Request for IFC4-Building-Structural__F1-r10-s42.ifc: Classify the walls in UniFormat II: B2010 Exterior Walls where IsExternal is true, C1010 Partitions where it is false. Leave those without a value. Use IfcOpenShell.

First a look at what the model holds.

```python
import ifcopenshell
import ifcopenshell.util.element

model = ifcopenshell.open("IFC4-Building-Structural__F1-r10-s42.ifc")
print(model.schema)
print("classifications:", [c.Name for c in model.by_type("IfcClassification")])
values = [ifcopenshell.util.element.get_pset(e, "Pset_WallCommon", "IsExternal") for e in model.by_type("IfcWall")]
for value in (True, False, None):
    print("IsExternal", value, values.count(value))
```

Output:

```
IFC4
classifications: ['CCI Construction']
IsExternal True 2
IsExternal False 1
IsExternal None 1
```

```python
import ifcopenshell
import ifcopenshell.api.classification
import ifcopenshell.util.element

model = ifcopenshell.open("IFC4-Building-Structural__F1-r10-s42.ifc")

system = ifcopenshell.api.classification.add_classification(model, classification="UniFormat II")

walls = model.by_type("IfcWall")
external = {e: ifcopenshell.util.element.get_pset(e, "Pset_WallCommon", "IsExternal") for e in walls}
for flag, code, name in ((True, "B2010", "Exterior Walls"), (False, "C1010", "Partitions")):
    products = [e for e in walls if external[e] is flag]
    ifcopenshell.api.classification.add_reference(
        model, products=products, classification=system, identification=code, name=name
    )
    print(code, len(products))

model.write("IFC4-Building-Structural__F1-r10-s42-out.ifc")
```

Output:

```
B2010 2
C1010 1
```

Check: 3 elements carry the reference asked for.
